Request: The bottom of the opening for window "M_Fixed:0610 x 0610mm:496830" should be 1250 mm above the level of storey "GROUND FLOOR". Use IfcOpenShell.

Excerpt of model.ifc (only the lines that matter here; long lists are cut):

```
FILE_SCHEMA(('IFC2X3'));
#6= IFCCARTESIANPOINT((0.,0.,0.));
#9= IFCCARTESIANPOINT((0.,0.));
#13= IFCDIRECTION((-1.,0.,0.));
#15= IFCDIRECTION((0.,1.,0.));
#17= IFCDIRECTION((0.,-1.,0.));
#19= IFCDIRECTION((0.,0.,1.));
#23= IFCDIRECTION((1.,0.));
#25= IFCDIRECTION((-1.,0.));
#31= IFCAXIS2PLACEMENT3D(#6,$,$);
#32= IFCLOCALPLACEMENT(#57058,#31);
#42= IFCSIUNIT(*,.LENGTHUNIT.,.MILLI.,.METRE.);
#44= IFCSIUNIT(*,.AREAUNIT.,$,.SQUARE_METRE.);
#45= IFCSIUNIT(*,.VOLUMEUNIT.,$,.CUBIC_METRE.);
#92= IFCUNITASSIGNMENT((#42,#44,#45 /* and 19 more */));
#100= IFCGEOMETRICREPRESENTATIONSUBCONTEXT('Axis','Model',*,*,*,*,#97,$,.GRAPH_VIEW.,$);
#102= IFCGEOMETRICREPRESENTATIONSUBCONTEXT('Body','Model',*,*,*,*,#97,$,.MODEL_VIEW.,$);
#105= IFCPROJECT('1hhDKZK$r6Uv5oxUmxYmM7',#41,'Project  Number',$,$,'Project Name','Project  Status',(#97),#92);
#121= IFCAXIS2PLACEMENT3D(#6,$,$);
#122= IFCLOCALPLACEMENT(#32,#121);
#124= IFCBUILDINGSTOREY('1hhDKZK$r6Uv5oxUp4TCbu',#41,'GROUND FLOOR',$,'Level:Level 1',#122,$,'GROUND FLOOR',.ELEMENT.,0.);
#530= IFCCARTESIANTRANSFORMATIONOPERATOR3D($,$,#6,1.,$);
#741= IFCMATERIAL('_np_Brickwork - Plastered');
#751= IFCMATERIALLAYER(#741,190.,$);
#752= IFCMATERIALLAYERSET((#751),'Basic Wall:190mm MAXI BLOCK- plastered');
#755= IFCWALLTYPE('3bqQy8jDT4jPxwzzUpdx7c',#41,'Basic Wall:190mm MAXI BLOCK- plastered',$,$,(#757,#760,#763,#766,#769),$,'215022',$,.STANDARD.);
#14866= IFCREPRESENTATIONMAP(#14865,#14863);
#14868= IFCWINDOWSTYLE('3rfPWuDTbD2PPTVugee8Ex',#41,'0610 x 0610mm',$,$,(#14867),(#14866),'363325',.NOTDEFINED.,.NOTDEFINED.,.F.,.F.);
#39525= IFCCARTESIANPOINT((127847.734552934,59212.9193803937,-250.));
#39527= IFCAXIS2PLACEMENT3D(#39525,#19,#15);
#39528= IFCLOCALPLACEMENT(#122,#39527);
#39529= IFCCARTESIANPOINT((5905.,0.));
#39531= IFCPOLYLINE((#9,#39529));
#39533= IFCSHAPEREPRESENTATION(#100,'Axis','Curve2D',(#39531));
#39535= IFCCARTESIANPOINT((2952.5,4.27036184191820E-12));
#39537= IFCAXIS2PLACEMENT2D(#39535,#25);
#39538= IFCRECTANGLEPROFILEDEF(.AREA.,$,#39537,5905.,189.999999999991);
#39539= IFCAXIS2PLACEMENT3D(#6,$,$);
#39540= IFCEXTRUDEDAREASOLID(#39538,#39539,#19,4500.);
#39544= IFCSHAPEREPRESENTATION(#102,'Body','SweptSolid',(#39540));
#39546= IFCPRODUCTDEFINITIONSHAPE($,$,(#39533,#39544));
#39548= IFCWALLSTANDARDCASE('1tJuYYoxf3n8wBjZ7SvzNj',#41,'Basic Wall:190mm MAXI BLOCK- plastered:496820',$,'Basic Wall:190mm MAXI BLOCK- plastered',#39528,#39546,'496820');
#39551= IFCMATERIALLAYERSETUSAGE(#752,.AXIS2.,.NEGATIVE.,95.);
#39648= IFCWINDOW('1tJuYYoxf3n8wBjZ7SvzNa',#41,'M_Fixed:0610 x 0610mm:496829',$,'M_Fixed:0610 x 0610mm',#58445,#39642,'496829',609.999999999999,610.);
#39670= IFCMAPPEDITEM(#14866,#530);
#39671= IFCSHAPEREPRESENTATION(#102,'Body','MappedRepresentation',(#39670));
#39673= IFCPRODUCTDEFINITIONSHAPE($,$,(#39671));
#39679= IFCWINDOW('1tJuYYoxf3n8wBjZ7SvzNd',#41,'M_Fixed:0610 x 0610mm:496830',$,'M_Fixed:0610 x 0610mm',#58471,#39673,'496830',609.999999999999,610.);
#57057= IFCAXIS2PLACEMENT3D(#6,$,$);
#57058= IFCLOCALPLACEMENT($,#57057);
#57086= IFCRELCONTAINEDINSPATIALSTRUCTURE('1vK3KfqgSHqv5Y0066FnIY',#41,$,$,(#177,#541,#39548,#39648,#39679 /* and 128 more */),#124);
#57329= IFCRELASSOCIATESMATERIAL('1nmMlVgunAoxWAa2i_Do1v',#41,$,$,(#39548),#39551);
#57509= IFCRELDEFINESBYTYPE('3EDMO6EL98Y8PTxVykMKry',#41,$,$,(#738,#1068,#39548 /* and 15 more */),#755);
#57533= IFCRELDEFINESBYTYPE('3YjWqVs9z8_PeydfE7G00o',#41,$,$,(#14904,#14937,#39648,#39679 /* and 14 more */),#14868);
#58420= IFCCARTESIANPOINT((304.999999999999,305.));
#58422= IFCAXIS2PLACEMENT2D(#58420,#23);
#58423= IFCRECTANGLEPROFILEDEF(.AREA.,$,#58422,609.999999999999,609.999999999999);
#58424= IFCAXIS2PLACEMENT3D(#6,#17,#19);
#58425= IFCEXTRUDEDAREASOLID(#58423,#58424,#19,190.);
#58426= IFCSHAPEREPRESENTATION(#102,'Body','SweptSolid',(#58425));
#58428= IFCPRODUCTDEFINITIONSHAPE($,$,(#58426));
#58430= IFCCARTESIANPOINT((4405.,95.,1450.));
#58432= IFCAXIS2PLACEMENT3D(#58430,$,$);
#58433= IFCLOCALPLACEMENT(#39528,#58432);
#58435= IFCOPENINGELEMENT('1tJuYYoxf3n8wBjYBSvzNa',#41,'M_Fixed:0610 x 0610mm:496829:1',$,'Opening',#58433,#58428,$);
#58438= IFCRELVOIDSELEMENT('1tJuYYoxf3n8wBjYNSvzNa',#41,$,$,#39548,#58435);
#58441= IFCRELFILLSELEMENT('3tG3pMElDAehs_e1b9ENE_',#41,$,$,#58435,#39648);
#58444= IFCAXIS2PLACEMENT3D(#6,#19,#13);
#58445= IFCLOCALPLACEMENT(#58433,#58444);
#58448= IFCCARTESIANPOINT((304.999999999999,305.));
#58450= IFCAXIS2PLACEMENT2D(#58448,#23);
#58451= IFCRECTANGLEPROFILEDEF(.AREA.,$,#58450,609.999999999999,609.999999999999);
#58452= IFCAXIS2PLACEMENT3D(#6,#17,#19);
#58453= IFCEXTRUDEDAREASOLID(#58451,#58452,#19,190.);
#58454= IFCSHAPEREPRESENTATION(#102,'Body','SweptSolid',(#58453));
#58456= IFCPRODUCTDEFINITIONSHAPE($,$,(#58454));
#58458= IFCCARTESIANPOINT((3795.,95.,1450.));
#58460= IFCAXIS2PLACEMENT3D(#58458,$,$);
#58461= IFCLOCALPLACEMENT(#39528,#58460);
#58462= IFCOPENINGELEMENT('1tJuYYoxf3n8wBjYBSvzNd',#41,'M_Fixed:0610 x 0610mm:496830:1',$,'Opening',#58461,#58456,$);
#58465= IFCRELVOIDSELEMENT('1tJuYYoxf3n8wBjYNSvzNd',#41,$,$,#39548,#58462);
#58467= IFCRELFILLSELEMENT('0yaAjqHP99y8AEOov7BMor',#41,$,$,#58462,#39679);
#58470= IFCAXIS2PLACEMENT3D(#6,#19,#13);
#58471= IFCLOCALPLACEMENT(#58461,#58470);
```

```python
import numpy as np
import ifcopenshell
import ifcopenshell.api.geometry
import ifcopenshell.geom
import ifcopenshell.util.element
import ifcopenshell.util.placement
import ifcopenshell.util.shape
import ifcopenshell.util.unit

model = ifcopenshell.open("model.ifc")
unit_scale = ifcopenshell.util.unit.calculate_unit_scale(model)

window = model.by_guid("1tJuYYoxf3n8wBjZ7SvzNd")
opening = window.FillsVoids[0].RelatingOpeningElement
storey = ifcopenshell.util.element.get_container(window, ifc_class="IfcBuildingStorey")
level = ifcopenshell.util.placement.get_local_placement(storey.ObjectPlacement)[2, 3]

# The opening's origin need not be at the sill, so measure its lowest point.
shape = ifcopenshell.geom.create_shape(ifcopenshell.geom.settings(), opening)
bottom = ifcopenshell.util.shape.get_shape_bottom_elevation(shape, shape.geometry) / unit_scale
dz = level + 1.25 / unit_scale - bottom

shift = np.array([0.0, 0.0, dz])
# The window is placed relative to its opening, so it follows when the opening moves.
matrix = ifcopenshell.util.placement.get_local_placement(opening.ObjectPlacement)
matrix[:3, 3] += shift
ifcopenshell.api.geometry.edit_object_placement(
    model, product=opening, matrix=matrix, is_si=False, should_transform_children=True
)

print(f"moved by {dz * unit_scale:+.3f} m")

model.write("model_rev.ifc")
```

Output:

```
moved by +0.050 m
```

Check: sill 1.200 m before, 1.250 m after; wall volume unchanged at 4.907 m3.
